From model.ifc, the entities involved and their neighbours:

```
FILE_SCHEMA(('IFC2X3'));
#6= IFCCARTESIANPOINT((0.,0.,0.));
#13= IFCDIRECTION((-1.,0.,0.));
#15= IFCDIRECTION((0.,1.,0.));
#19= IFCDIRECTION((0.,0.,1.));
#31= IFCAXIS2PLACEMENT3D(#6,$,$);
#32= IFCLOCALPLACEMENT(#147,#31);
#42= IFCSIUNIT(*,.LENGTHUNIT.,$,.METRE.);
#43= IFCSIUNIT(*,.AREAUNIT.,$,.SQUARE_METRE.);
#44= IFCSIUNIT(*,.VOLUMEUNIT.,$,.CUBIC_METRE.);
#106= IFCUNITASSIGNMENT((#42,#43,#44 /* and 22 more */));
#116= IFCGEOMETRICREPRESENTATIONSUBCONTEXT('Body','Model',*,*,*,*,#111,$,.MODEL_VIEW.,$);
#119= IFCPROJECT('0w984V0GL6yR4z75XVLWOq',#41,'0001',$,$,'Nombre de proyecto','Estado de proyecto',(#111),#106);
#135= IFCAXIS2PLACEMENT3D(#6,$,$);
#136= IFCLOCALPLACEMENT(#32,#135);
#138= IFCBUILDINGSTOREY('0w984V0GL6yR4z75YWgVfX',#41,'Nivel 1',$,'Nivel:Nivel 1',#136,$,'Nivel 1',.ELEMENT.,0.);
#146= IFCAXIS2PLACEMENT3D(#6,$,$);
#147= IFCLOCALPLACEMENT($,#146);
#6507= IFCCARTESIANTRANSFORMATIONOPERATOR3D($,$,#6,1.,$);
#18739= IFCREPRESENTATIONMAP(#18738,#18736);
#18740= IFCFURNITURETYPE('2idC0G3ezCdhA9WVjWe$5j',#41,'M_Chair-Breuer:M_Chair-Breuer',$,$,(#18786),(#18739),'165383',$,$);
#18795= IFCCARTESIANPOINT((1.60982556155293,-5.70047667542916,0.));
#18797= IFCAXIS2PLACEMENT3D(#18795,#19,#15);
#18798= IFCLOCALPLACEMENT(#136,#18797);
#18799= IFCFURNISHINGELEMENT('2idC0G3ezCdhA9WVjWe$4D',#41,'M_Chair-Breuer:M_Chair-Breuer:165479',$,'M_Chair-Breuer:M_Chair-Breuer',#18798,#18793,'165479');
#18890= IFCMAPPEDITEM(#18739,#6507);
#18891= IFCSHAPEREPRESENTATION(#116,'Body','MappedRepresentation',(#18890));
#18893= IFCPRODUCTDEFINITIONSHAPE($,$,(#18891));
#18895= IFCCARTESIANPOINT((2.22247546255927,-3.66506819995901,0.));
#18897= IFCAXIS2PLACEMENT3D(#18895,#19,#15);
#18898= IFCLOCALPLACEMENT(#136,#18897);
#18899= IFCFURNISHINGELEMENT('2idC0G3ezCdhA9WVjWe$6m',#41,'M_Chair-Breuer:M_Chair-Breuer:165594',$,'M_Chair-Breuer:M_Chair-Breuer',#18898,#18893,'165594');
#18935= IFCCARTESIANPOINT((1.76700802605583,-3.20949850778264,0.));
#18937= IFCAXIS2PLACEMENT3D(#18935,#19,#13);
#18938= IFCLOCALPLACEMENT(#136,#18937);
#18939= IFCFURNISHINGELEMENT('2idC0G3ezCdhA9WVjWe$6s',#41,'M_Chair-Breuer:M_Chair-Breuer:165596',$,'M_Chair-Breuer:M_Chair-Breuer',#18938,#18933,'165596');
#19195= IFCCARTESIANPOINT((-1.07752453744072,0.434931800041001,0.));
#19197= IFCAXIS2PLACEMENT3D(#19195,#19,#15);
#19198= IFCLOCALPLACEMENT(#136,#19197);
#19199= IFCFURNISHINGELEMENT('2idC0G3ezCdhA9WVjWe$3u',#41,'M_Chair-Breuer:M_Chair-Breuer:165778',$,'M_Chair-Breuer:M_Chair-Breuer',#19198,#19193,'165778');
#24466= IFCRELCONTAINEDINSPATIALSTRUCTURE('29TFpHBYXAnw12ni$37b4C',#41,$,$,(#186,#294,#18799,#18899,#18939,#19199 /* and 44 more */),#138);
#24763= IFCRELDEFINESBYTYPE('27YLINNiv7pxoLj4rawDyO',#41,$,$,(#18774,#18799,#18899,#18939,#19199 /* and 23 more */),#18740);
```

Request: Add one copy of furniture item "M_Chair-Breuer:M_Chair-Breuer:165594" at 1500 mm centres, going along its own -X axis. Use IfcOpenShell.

```python
import ifcopenshell
import ifcopenshell.api.geometry
import ifcopenshell.api.root
import ifcopenshell.util.element
import ifcopenshell.util.placement

model = ifcopenshell.open("model.ifc")


def reuse_history(source, copy):
    """copy_class also copies each property set's owner history, people and application; keep the originals."""
    for rel in copy.IsDefinedBy:
        if rel.is_a("IfcRelDefinesByProperties") and (history := rel.RelatingPropertyDefinition.OwnerHistory):
            rel.RelatingPropertyDefinition.OwnerHistory = source.OwnerHistory
            ifcopenshell.util.element.remove_deep2(model, history)


source = model.by_guid("2idC0G3ezCdhA9WVjWe$6m")
base = ifcopenshell.util.placement.get_local_placement(source.ObjectPlacement)
step = -base[:3, 0] * 1.5

for i in range(1, 2):
    copy = ifcopenshell.api.root.copy_class(model, product=source)
    copy.Representation = ifcopenshell.util.element.copy_deep(
        model, source.Representation, exclude=["IfcGeometricRepresentationContext", "IfcRepresentationMap"]
    )
    copy.Name = "M_Chair-Breuer:M_Chair-Breuer"
    copy.Tag = None
    reuse_history(source, copy)
    matrix = base.copy()
    matrix[:3, 3] += i * step
    print("added at", matrix[:3, 3].round(3) + 0.0)
    ifcopenshell.api.geometry.edit_object_placement(model, product=copy, matrix=matrix, is_si=False)

model.write("model_edited.ifc")
```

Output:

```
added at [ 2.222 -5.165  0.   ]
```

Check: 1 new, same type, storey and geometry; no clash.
